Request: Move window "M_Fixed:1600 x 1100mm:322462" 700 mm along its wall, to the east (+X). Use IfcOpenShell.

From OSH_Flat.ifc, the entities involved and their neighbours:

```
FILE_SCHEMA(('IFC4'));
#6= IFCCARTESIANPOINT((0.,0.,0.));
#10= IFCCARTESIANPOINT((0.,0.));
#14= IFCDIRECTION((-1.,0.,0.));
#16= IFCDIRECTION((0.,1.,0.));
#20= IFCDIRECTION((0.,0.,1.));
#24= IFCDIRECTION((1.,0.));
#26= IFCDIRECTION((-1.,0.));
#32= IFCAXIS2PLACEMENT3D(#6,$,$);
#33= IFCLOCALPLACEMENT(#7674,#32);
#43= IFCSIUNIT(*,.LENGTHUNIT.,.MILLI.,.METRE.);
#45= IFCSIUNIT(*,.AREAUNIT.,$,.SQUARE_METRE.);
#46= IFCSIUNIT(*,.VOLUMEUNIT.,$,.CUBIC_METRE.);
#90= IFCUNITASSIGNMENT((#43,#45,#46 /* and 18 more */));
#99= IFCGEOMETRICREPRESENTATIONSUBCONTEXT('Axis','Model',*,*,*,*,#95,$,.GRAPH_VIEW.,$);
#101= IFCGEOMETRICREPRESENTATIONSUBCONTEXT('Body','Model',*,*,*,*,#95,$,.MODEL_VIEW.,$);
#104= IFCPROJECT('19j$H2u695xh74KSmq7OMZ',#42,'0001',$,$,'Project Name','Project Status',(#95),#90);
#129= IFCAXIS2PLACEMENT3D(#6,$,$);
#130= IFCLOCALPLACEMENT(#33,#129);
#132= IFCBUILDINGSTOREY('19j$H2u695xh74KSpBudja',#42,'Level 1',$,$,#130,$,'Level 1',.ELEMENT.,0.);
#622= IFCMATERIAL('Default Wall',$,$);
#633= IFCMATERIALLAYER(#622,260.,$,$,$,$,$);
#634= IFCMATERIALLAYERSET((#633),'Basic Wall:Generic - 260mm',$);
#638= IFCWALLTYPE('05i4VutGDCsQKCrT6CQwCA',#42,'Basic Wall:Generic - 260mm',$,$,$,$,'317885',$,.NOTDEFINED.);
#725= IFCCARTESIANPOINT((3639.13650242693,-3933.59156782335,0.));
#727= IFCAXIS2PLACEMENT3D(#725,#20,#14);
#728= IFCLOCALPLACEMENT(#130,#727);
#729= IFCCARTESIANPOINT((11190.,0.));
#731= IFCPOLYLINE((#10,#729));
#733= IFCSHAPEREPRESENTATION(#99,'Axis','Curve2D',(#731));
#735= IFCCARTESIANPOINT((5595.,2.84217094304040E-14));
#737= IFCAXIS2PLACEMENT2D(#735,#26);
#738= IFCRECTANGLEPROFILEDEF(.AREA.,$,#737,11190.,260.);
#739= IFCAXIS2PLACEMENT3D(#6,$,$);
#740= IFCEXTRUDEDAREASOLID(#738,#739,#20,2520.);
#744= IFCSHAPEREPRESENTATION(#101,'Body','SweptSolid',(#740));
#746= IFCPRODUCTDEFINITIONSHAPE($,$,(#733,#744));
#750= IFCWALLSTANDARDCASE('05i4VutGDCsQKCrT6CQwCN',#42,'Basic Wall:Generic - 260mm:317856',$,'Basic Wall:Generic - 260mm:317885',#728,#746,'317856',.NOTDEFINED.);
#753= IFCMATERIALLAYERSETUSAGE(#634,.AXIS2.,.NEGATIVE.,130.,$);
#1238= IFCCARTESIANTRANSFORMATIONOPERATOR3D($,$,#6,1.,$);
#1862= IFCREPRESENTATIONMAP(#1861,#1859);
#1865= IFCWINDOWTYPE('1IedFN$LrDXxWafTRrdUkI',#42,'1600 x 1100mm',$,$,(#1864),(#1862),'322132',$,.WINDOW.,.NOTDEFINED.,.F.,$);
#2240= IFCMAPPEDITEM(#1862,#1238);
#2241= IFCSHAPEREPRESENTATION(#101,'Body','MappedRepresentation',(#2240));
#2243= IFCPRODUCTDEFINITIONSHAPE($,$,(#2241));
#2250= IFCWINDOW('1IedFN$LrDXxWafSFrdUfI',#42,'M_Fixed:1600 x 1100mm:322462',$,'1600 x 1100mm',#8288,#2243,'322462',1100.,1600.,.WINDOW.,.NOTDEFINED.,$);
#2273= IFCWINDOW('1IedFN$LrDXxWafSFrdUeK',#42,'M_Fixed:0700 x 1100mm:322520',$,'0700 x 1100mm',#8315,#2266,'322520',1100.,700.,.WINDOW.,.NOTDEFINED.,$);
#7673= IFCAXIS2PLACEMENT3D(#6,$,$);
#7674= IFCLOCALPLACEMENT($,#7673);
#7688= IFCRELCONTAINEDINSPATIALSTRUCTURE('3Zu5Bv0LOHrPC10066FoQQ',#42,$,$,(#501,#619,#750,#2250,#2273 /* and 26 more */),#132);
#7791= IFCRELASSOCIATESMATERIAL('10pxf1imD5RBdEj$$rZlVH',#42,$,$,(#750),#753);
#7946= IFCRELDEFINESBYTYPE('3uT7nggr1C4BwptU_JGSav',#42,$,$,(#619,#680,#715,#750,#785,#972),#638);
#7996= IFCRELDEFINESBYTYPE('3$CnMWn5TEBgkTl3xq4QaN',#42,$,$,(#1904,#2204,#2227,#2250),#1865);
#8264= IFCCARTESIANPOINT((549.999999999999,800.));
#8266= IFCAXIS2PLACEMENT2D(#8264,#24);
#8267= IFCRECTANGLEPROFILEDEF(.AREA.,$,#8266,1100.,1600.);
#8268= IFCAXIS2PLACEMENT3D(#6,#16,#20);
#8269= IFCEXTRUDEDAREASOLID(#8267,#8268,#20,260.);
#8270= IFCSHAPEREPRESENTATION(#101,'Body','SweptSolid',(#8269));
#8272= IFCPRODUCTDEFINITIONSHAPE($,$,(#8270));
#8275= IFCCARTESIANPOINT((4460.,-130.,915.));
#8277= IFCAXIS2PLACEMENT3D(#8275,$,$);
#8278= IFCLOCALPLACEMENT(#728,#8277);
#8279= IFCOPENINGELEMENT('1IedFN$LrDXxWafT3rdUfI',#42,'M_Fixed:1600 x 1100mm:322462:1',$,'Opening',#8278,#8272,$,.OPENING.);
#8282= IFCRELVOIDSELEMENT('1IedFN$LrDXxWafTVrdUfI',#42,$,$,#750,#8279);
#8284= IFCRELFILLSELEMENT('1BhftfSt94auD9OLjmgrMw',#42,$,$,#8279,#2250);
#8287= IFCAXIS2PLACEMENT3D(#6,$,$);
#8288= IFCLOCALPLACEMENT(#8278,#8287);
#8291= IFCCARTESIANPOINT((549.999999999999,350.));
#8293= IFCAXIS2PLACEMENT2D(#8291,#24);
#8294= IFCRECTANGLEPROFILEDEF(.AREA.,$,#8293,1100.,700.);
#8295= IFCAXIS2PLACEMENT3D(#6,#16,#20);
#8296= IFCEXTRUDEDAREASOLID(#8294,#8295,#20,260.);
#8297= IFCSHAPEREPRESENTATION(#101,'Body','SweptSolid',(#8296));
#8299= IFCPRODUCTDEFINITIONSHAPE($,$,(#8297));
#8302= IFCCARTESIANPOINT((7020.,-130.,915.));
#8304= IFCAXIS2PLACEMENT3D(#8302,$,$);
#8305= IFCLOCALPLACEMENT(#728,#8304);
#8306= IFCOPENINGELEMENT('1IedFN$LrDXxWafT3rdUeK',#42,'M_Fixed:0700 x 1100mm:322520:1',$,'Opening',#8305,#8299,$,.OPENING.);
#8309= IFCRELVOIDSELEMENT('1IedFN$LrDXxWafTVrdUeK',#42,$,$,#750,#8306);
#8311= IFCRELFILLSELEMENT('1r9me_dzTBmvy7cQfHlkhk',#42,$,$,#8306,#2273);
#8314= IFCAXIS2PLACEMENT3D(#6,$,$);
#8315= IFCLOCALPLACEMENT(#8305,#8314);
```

```python
import ifcopenshell
import ifcopenshell.api.geometry
import ifcopenshell.util.placement

model = ifcopenshell.open("OSH_Flat.ifc")

window = model.by_guid("1IedFN$LrDXxWafSFrdUfI")
opening = window.FillsVoids[0].RelatingOpeningElement
wall = opening.VoidsElements[0].RelatingBuildingElement

wall_matrix = ifcopenshell.util.placement.get_local_placement(wall.ObjectPlacement)
shift = wall_matrix[:3, 0] * -700.0
before = ifcopenshell.util.placement.get_local_placement(window.ObjectPlacement)[:3, 3].copy()

# The window is placed relative to its opening, so it follows when the opening moves.
matrix = ifcopenshell.util.placement.get_local_placement(opening.ObjectPlacement)
matrix[:3, 3] += shift
ifcopenshell.api.geometry.edit_object_placement(
    model, product=opening, matrix=matrix, is_si=False, should_transform_children=True
)

after = ifcopenshell.util.placement.get_local_placement(window.ObjectPlacement)[:3, 3]
print("window moved by", (after - before).round(3) + 0.0)

model.write("OSH_Flat_rev.ifc")
```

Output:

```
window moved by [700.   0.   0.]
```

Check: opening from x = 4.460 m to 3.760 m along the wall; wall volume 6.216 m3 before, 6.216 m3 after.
